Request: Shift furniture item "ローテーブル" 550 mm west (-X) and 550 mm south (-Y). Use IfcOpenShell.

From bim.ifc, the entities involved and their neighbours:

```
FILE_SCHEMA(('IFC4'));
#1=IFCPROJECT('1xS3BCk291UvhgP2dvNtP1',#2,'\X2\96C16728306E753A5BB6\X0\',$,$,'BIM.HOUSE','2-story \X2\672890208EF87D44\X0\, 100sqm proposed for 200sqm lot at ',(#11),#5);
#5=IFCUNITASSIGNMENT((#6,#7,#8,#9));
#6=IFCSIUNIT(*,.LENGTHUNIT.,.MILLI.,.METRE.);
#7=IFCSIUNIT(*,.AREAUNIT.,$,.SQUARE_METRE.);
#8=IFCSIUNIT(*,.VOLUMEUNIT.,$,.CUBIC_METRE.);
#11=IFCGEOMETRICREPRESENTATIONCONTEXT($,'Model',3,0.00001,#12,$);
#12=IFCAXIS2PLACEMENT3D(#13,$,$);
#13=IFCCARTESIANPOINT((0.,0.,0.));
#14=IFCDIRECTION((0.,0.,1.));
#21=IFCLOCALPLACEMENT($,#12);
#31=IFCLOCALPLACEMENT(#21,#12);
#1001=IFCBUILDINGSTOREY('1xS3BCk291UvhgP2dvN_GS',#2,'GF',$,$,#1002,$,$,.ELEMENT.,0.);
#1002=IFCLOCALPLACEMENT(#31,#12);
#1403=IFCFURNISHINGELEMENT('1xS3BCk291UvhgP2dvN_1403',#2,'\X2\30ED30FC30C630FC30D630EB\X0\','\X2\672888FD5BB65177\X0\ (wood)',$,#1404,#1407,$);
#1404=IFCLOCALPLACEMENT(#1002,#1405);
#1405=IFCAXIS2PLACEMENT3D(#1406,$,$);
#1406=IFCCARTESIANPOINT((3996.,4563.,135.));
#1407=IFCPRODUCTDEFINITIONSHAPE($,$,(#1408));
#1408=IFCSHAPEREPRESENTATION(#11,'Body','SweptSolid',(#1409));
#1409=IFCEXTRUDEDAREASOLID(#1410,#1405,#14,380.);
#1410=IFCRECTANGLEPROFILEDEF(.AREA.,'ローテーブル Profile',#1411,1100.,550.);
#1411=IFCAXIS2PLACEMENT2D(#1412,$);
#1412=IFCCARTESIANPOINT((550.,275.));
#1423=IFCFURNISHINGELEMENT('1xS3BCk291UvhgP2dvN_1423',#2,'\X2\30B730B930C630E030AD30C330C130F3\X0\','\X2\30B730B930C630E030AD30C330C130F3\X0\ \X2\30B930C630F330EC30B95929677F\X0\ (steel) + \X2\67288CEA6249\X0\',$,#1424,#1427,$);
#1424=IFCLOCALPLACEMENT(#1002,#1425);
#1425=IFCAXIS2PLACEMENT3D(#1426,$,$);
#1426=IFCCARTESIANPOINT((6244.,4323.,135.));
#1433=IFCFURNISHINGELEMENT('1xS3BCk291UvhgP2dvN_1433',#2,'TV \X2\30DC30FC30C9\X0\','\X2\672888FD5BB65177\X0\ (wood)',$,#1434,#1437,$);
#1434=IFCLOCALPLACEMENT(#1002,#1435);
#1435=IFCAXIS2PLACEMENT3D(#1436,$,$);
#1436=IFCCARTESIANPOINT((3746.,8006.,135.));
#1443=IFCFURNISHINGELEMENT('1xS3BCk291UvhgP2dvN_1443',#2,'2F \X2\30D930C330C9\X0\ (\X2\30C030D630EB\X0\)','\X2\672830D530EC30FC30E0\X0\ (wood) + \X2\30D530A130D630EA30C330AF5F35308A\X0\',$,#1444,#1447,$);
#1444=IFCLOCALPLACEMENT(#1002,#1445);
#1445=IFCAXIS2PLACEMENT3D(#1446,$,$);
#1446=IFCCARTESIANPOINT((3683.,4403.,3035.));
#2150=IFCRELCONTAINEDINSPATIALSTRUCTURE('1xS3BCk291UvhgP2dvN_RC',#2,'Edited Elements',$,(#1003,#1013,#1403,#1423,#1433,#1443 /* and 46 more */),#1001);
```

```python
import ifcopenshell
import ifcopenshell.api.geometry
import ifcopenshell.util.placement
import ifcopenshell.util.unit

model = ifcopenshell.open("bim.ifc")
unit_scale = ifcopenshell.util.unit.calculate_unit_scale(model)

item = model.by_guid("1xS3BCk291UvhgP2dvN_1403")
matrix = ifcopenshell.util.placement.get_local_placement(item.ObjectPlacement)
matrix[0, 3] -= 0.55 / unit_scale
matrix[1, 3] -= 0.55 / unit_scale
ifcopenshell.api.geometry.edit_object_placement(model, product=item, matrix=matrix, is_si=False)

print(ifcopenshell.util.placement.get_local_placement(item.ObjectPlacement).round(3) + 0.0)

model.write("bim_v2.ifc")
```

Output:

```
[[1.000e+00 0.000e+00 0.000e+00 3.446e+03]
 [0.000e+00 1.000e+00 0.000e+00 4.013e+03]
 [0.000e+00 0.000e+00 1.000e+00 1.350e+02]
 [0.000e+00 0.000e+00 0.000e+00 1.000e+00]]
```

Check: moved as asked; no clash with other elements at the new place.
